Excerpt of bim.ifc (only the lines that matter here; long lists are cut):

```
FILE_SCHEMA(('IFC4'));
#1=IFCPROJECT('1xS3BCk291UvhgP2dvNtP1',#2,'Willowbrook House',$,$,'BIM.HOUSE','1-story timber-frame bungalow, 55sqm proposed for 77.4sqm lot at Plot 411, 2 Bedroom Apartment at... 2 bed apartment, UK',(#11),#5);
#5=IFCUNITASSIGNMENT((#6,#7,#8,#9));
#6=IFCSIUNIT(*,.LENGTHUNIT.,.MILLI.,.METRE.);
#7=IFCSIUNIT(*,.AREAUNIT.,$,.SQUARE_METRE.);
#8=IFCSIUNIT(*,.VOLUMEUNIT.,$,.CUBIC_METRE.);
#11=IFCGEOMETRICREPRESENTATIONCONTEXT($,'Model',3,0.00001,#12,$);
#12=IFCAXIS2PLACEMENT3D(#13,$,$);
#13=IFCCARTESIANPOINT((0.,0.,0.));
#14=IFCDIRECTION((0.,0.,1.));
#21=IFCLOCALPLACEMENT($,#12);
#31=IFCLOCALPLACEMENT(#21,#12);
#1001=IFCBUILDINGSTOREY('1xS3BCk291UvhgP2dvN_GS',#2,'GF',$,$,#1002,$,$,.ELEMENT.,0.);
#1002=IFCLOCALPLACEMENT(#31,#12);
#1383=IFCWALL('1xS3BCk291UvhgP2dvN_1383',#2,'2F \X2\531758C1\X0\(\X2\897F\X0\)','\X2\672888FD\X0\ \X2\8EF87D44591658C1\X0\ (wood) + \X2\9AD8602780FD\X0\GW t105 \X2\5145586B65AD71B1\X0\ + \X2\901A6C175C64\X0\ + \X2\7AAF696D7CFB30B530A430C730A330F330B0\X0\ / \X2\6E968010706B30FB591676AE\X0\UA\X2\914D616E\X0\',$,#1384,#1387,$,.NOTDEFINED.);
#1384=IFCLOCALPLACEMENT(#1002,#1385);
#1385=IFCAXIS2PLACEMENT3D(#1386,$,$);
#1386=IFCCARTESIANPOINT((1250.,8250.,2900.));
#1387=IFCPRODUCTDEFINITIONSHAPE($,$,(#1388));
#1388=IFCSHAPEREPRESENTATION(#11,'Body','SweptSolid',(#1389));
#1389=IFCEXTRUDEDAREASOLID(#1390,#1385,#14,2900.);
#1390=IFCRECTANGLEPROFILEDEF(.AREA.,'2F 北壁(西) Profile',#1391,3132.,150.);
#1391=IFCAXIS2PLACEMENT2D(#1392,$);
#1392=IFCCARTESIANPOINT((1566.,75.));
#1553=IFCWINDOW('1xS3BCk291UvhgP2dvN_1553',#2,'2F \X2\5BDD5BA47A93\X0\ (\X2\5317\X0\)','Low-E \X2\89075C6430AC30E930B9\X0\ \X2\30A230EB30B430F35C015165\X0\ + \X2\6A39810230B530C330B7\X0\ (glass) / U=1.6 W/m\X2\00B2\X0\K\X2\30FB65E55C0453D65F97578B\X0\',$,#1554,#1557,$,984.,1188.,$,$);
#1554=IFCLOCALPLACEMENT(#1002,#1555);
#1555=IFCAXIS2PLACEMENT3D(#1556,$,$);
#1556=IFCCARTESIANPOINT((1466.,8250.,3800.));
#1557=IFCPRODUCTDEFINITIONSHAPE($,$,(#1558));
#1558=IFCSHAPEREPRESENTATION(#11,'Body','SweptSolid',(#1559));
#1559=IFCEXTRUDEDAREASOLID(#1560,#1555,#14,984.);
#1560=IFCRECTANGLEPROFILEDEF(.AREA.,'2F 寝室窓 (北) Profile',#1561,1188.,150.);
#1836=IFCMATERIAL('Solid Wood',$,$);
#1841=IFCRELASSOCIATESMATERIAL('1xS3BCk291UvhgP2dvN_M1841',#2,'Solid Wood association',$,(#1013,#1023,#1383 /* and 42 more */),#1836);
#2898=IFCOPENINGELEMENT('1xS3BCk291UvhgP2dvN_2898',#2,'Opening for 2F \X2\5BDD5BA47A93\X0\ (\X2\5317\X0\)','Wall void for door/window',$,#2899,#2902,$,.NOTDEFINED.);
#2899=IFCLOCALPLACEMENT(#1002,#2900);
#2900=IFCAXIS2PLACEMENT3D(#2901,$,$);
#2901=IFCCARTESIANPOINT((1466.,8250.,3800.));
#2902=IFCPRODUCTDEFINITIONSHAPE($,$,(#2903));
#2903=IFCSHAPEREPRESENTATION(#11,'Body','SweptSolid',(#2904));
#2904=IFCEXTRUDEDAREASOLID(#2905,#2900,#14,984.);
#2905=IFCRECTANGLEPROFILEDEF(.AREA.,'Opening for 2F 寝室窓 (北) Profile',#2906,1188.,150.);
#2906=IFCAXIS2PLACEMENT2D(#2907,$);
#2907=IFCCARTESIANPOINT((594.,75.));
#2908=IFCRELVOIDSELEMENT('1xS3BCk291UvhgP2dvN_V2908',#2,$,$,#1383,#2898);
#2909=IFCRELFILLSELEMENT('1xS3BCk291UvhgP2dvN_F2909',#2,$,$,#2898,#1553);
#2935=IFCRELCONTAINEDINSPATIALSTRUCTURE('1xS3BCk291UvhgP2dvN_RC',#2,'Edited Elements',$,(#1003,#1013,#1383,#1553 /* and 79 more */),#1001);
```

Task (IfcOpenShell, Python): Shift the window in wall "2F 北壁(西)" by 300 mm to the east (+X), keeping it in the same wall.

```python
import ifcopenshell
import ifcopenshell.api.geometry
import ifcopenshell.util.placement

model = ifcopenshell.open("bim.ifc")

window = model.by_id(1553)
opening = window.FillsVoids[0].RelatingOpeningElement
wall = opening.VoidsElements[0].RelatingBuildingElement

wall_matrix = ifcopenshell.util.placement.get_local_placement(wall.ObjectPlacement)
shift = wall_matrix[:3, 0] * 300.0
before = ifcopenshell.util.placement.get_local_placement(window.ObjectPlacement)[:3, 3].copy()

# The window is not placed relative to its opening, so move both.
for product in (opening, window):
    matrix = ifcopenshell.util.placement.get_local_placement(product.ObjectPlacement)
    matrix[:3, 3] += shift
    ifcopenshell.api.geometry.edit_object_placement(model, product=product, matrix=matrix, is_si=False)

after = ifcopenshell.util.placement.get_local_placement(window.ObjectPlacement)[:3, 3]
print("window moved by", (after - before).round(3) + 0.0)

model.write("bim_rev.ifc")
```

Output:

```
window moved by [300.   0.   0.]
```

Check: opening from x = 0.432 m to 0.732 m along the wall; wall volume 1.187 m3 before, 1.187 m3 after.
